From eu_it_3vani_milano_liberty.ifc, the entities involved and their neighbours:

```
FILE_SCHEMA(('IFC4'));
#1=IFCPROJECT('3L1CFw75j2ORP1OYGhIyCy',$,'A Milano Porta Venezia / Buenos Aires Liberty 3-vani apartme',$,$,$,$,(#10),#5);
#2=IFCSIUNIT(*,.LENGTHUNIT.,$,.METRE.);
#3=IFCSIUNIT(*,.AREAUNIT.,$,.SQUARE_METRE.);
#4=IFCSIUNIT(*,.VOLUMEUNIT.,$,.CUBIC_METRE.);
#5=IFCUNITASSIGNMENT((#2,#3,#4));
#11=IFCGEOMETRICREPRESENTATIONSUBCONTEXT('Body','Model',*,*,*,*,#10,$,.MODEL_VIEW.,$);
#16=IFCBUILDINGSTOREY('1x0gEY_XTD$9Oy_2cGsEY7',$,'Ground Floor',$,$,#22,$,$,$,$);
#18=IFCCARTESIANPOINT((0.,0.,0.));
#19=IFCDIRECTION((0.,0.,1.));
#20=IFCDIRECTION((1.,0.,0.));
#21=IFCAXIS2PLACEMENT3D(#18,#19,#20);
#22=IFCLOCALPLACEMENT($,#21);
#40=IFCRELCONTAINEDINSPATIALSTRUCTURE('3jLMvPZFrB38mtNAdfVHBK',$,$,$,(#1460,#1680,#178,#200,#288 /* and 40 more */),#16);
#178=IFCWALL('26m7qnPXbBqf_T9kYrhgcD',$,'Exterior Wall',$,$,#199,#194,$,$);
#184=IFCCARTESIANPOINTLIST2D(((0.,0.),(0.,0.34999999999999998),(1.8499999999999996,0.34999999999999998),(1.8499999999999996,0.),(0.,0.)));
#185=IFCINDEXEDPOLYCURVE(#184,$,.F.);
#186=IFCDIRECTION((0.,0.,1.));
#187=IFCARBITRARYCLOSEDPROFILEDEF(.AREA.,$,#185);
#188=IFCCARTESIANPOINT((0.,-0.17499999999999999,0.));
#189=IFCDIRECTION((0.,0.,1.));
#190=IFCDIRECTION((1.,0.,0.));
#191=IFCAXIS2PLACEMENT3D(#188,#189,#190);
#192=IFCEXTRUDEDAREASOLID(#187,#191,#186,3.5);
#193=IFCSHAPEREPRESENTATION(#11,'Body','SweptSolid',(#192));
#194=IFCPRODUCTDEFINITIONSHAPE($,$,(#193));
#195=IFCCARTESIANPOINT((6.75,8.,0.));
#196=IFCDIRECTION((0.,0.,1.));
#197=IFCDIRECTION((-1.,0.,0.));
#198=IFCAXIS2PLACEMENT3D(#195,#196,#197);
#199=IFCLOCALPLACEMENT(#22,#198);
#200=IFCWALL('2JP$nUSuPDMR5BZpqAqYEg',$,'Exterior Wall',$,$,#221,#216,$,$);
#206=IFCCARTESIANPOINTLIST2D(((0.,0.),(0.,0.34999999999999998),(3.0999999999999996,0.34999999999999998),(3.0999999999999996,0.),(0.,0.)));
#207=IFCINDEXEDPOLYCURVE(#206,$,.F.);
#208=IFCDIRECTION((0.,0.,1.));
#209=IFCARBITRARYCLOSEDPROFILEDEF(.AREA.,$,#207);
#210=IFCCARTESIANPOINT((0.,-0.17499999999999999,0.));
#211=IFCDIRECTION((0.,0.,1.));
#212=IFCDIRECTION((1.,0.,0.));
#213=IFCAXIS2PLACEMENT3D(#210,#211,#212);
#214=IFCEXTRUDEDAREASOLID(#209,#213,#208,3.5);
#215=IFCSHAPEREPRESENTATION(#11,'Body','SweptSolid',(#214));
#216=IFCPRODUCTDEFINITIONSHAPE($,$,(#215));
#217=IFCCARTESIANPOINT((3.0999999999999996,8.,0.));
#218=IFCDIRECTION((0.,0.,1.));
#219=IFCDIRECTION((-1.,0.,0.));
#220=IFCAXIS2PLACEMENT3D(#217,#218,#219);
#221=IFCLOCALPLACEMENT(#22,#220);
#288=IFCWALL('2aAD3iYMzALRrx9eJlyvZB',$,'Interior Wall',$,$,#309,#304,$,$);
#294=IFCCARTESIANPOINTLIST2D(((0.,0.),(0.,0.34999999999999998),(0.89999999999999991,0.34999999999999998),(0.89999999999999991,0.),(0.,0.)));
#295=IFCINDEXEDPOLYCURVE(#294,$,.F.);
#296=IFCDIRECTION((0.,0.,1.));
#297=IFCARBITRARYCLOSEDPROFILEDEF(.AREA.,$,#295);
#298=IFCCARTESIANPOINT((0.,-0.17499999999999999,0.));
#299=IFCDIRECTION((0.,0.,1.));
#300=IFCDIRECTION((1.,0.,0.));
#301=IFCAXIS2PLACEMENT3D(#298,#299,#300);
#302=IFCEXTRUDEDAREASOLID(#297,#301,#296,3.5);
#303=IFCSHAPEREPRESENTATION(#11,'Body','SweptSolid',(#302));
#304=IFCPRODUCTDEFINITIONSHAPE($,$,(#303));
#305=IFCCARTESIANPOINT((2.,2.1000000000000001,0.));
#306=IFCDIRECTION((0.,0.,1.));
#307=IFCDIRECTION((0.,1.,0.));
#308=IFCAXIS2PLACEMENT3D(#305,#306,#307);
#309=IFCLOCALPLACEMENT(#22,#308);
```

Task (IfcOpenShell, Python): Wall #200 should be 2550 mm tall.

```python
import ifcopenshell
import ifcopenshell.geom
import ifcopenshell.util.representation
import ifcopenshell.util.shape

model = ifcopenshell.open("eu_it_3vani_milano_liberty.ifc")
settings = ifcopenshell.geom.settings()


def volume(element):
    """Net volume in cubic metres, openings subtracted."""
    shape = ifcopenshell.geom.create_shape(settings, element)
    return ifcopenshell.util.shape.get_volume(shape.geometry)


wall = model.by_guid("2JP$nUSuPDMR5BZpqAqYEg")
before = volume(wall)

body = ifcopenshell.util.representation.get_representation(wall, "Model", "Body")
solid = body.Items[0]
old_height = solid.Depth
solid.Depth = 2.55
after = volume(wall)

print(f"height {old_height:g} -> {solid.Depth:g}, volume {before:.3f} -> {after:.3f} m3")

model.write("eu_it_3vani_milano_liberty_rev.ifc")
```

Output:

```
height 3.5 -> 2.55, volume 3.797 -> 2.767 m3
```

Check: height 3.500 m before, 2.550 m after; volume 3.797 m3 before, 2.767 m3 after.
